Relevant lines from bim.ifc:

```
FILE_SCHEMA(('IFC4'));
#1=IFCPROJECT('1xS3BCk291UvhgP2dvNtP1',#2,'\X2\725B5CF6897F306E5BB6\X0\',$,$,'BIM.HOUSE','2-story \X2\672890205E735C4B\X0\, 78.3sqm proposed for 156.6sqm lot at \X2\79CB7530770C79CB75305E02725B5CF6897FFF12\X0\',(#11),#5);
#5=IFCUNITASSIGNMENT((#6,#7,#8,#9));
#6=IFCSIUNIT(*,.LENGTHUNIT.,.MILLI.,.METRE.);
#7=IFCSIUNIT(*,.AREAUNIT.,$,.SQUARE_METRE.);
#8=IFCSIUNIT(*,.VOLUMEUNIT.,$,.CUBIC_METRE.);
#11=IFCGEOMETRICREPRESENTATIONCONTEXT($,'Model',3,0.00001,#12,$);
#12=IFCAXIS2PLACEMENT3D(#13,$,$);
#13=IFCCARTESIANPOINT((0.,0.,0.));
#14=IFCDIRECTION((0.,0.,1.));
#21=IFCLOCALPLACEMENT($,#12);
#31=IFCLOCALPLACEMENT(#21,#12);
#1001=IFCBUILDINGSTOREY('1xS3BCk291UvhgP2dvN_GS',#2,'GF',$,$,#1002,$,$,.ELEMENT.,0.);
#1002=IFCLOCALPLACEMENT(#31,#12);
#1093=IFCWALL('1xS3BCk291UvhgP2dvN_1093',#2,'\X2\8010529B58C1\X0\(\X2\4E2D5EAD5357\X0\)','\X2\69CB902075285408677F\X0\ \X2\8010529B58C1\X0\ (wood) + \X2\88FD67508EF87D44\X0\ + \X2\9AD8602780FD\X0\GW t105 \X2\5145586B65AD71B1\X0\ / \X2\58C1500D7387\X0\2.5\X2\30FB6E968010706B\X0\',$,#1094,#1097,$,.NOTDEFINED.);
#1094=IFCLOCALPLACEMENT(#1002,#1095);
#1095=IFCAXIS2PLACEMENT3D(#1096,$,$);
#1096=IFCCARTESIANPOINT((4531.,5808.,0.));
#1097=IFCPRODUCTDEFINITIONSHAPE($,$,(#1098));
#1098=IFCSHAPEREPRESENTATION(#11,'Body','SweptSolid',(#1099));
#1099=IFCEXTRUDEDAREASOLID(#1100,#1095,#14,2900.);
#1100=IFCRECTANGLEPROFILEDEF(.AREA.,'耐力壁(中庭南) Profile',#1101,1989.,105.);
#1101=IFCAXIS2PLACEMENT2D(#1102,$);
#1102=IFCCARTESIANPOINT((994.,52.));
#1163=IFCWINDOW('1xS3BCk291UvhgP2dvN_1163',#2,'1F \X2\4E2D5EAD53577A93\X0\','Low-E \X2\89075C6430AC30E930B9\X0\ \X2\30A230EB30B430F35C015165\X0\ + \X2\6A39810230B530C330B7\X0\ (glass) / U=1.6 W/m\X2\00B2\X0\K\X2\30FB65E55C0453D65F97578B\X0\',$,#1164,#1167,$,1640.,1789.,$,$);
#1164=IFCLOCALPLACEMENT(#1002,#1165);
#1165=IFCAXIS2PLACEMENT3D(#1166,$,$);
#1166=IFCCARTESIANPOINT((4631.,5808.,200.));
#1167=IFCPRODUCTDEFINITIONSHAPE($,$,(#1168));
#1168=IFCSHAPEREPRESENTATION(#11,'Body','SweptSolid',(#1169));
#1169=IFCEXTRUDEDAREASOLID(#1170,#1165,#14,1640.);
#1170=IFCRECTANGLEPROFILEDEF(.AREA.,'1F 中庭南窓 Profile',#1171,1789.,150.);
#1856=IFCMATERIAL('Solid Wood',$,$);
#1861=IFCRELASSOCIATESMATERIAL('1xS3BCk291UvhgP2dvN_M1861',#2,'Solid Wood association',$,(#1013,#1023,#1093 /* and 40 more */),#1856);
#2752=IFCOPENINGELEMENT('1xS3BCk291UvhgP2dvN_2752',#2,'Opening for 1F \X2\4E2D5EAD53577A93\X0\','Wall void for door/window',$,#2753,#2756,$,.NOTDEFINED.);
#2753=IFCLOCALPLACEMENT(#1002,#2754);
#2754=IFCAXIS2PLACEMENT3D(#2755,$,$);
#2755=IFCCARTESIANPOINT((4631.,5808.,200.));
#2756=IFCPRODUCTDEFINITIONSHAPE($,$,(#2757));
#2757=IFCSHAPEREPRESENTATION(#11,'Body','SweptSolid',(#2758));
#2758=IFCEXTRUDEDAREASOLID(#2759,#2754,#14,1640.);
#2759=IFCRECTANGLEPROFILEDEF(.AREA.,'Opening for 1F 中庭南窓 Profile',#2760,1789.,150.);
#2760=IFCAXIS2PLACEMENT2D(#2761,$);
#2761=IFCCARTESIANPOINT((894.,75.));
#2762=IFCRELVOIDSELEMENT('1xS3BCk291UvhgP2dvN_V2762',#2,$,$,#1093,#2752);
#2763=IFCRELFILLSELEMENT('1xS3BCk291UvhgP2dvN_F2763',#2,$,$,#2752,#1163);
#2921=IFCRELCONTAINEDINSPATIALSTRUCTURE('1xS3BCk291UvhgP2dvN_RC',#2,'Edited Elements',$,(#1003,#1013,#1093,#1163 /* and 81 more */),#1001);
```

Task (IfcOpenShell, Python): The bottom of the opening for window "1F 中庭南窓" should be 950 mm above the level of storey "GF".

```python
import numpy as np
import ifcopenshell
import ifcopenshell.api.geometry
import ifcopenshell.geom
import ifcopenshell.util.element
import ifcopenshell.util.placement
import ifcopenshell.util.shape
import ifcopenshell.util.unit

model = ifcopenshell.open("bim.ifc")
unit_scale = ifcopenshell.util.unit.calculate_unit_scale(model)

window = model.by_id(1163)
opening = window.FillsVoids[0].RelatingOpeningElement
storey = ifcopenshell.util.element.get_container(window, ifc_class="IfcBuildingStorey")
level = ifcopenshell.util.placement.get_local_placement(storey.ObjectPlacement)[2, 3]

# The opening's origin need not be at the sill, so measure its lowest point.
shape = ifcopenshell.geom.create_shape(ifcopenshell.geom.settings(), opening)
bottom = ifcopenshell.util.shape.get_shape_bottom_elevation(shape, shape.geometry) / unit_scale
dz = level + 950.0 - bottom

shift = np.array([0.0, 0.0, dz])
# The window is not placed relative to its opening, so move both.
for product in (opening, window):
    matrix = ifcopenshell.util.placement.get_local_placement(product.ObjectPlacement)
    matrix[:3, 3] += shift
    ifcopenshell.api.geometry.edit_object_placement(model, product=product, matrix=matrix, is_si=False)

print(f"moved by {dz * unit_scale:+.3f} m")

model.write("bim-out.ifc")
```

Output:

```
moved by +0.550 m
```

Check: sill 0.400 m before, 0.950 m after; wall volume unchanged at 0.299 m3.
